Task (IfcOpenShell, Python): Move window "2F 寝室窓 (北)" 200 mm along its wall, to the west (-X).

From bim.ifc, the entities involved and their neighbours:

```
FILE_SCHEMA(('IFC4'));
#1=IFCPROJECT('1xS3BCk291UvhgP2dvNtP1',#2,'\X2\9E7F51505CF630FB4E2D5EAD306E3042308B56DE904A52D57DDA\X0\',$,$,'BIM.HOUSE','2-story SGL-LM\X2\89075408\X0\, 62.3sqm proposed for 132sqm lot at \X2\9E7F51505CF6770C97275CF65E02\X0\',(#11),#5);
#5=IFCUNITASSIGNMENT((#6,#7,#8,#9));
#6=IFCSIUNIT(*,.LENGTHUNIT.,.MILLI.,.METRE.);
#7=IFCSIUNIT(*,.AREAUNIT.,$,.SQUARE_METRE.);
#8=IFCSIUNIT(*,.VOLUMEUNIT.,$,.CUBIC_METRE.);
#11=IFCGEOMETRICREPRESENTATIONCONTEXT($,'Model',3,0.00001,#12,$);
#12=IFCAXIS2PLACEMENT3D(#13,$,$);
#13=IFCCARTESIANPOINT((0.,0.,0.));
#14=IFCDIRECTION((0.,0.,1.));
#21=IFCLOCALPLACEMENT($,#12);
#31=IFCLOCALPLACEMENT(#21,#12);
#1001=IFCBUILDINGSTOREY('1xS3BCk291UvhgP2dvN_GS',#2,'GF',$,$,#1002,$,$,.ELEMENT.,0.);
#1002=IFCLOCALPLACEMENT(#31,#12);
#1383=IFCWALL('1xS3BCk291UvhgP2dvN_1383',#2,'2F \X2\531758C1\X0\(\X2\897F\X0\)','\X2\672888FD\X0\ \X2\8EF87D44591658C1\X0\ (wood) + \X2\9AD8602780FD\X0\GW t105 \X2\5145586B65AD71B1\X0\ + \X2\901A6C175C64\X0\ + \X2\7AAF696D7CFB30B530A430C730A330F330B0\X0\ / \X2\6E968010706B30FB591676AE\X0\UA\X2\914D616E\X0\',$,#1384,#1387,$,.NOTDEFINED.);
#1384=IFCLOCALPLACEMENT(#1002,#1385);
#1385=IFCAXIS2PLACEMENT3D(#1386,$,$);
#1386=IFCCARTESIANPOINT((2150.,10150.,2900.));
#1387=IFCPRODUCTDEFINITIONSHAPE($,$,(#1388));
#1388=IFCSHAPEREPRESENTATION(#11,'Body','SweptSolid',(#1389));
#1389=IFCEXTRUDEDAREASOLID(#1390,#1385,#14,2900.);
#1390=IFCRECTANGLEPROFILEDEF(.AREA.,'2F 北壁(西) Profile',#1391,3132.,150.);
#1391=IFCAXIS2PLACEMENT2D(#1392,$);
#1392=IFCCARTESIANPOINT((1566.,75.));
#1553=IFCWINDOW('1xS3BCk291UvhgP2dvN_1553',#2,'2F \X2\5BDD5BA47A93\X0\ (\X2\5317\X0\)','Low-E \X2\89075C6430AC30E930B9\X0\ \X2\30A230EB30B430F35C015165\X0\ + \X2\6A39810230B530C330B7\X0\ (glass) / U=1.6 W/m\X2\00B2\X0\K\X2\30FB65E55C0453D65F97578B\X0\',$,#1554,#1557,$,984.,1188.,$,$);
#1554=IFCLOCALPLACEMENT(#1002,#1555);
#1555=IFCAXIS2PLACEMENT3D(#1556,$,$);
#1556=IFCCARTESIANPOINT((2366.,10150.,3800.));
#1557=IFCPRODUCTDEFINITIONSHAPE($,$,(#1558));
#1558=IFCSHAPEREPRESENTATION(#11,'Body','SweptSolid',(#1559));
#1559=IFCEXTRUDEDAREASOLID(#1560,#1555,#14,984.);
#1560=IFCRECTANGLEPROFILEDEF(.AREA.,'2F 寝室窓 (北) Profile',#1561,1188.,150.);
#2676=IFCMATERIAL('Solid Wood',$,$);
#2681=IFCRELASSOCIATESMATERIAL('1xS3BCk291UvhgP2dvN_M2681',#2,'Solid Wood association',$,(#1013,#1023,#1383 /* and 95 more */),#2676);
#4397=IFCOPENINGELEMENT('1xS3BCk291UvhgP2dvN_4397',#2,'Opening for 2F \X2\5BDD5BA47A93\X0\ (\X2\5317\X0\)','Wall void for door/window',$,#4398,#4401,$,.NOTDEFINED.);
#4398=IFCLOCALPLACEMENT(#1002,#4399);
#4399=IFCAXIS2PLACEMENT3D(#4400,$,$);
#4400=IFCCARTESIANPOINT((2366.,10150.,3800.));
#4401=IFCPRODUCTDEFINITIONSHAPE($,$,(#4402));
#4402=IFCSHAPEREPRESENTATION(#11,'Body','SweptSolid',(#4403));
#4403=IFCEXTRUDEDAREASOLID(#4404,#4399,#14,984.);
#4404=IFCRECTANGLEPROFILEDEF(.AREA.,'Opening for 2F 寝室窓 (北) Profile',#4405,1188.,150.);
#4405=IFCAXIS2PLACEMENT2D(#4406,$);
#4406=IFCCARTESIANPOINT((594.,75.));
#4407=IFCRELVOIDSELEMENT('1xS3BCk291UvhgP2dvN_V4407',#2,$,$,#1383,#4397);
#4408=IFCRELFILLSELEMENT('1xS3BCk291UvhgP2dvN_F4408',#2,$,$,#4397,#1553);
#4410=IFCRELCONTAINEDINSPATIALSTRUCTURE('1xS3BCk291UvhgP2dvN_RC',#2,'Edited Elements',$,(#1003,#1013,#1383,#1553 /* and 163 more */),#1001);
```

```python
import ifcopenshell
import ifcopenshell.api.geometry
import ifcopenshell.util.placement
import ifcopenshell.util.unit

model = ifcopenshell.open("bim.ifc")
unit_scale = ifcopenshell.util.unit.calculate_unit_scale(model)

window = model.by_id(1553)
opening = window.FillsVoids[0].RelatingOpeningElement
wall = opening.VoidsElements[0].RelatingBuildingElement

wall_matrix = ifcopenshell.util.placement.get_local_placement(wall.ObjectPlacement)
shift = wall_matrix[:3, 0] * -0.2 / unit_scale
before = ifcopenshell.util.placement.get_local_placement(window.ObjectPlacement)[:3, 3].copy()

# The window is not placed relative to its opening, so move both.
for product in (opening, window):
    matrix = ifcopenshell.util.placement.get_local_placement(product.ObjectPlacement)
    matrix[:3, 3] += shift
    ifcopenshell.api.geometry.edit_object_placement(model, product=product, matrix=matrix, is_si=False)

after = ifcopenshell.util.placement.get_local_placement(window.ObjectPlacement)[:3, 3]
print("window moved by", (after - before).round(3) + 0.0)

model.write("bim_updated.ifc")
```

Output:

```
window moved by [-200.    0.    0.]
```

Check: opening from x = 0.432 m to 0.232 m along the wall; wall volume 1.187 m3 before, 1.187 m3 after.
